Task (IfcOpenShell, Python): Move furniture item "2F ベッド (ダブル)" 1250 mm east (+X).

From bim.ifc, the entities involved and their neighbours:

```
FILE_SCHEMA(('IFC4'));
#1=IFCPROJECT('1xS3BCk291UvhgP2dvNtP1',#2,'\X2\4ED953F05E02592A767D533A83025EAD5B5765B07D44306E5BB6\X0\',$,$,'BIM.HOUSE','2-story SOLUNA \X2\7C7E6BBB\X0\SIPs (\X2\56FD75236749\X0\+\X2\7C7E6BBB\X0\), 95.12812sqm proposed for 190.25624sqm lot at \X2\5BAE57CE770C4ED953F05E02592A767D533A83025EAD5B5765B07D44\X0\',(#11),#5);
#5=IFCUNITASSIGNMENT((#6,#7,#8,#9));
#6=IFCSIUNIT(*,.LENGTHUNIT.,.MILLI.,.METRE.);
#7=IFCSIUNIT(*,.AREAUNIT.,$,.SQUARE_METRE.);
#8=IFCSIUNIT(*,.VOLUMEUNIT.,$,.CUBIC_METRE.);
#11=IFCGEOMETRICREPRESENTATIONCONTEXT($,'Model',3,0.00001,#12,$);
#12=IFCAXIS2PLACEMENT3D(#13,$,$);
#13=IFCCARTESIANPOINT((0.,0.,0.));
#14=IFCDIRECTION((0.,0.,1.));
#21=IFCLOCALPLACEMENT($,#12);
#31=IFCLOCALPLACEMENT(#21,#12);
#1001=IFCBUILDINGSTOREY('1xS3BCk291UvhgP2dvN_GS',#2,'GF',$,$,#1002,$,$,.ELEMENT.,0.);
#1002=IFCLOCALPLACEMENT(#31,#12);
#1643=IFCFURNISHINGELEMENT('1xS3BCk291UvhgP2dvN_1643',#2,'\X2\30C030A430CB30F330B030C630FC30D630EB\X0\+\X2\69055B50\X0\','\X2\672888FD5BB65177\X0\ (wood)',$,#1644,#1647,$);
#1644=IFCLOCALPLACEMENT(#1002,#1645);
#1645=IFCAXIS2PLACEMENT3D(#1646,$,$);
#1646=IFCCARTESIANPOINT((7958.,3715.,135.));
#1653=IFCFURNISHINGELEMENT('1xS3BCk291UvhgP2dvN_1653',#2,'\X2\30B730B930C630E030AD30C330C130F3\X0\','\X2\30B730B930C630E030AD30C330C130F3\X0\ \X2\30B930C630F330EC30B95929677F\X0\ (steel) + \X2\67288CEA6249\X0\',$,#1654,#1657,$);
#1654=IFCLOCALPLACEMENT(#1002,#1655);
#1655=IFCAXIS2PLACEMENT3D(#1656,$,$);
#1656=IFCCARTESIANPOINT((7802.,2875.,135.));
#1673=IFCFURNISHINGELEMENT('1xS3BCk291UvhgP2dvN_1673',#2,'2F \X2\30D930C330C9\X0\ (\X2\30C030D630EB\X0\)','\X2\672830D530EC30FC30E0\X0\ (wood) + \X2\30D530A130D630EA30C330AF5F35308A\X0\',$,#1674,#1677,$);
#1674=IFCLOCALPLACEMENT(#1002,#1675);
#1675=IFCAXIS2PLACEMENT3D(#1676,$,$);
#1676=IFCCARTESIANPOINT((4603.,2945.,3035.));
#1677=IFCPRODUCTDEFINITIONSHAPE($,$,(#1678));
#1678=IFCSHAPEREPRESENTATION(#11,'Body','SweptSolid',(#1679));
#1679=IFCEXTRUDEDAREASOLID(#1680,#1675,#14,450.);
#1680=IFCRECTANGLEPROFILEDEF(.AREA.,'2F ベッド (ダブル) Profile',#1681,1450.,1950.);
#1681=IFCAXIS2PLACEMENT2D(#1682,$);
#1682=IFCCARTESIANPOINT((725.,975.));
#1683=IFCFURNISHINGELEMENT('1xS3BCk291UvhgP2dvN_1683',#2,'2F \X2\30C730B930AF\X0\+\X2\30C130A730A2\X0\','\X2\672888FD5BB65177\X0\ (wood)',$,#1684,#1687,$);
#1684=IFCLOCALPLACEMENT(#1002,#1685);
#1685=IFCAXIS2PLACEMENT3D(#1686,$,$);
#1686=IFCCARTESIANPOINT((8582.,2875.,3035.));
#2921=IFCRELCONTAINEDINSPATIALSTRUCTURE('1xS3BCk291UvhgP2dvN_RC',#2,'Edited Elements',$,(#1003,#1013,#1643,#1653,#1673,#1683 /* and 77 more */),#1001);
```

```python
import ifcopenshell
import ifcopenshell.api.geometry
import ifcopenshell.util.placement
import ifcopenshell.util.unit

model = ifcopenshell.open("bim.ifc")
unit_scale = ifcopenshell.util.unit.calculate_unit_scale(model)

item = model.by_guid("1xS3BCk291UvhgP2dvN_1673")
matrix = ifcopenshell.util.placement.get_local_placement(item.ObjectPlacement)
matrix[0, 3] += 1.25 / unit_scale
ifcopenshell.api.geometry.edit_object_placement(model, product=item, matrix=matrix, is_si=False)

print(ifcopenshell.util.placement.get_local_placement(item.ObjectPlacement).round(3) + 0.0)

model.write("bim_v2.ifc")
```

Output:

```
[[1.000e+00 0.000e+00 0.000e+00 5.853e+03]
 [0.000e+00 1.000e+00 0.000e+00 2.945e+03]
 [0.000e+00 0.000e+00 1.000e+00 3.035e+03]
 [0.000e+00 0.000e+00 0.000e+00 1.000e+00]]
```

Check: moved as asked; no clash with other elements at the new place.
